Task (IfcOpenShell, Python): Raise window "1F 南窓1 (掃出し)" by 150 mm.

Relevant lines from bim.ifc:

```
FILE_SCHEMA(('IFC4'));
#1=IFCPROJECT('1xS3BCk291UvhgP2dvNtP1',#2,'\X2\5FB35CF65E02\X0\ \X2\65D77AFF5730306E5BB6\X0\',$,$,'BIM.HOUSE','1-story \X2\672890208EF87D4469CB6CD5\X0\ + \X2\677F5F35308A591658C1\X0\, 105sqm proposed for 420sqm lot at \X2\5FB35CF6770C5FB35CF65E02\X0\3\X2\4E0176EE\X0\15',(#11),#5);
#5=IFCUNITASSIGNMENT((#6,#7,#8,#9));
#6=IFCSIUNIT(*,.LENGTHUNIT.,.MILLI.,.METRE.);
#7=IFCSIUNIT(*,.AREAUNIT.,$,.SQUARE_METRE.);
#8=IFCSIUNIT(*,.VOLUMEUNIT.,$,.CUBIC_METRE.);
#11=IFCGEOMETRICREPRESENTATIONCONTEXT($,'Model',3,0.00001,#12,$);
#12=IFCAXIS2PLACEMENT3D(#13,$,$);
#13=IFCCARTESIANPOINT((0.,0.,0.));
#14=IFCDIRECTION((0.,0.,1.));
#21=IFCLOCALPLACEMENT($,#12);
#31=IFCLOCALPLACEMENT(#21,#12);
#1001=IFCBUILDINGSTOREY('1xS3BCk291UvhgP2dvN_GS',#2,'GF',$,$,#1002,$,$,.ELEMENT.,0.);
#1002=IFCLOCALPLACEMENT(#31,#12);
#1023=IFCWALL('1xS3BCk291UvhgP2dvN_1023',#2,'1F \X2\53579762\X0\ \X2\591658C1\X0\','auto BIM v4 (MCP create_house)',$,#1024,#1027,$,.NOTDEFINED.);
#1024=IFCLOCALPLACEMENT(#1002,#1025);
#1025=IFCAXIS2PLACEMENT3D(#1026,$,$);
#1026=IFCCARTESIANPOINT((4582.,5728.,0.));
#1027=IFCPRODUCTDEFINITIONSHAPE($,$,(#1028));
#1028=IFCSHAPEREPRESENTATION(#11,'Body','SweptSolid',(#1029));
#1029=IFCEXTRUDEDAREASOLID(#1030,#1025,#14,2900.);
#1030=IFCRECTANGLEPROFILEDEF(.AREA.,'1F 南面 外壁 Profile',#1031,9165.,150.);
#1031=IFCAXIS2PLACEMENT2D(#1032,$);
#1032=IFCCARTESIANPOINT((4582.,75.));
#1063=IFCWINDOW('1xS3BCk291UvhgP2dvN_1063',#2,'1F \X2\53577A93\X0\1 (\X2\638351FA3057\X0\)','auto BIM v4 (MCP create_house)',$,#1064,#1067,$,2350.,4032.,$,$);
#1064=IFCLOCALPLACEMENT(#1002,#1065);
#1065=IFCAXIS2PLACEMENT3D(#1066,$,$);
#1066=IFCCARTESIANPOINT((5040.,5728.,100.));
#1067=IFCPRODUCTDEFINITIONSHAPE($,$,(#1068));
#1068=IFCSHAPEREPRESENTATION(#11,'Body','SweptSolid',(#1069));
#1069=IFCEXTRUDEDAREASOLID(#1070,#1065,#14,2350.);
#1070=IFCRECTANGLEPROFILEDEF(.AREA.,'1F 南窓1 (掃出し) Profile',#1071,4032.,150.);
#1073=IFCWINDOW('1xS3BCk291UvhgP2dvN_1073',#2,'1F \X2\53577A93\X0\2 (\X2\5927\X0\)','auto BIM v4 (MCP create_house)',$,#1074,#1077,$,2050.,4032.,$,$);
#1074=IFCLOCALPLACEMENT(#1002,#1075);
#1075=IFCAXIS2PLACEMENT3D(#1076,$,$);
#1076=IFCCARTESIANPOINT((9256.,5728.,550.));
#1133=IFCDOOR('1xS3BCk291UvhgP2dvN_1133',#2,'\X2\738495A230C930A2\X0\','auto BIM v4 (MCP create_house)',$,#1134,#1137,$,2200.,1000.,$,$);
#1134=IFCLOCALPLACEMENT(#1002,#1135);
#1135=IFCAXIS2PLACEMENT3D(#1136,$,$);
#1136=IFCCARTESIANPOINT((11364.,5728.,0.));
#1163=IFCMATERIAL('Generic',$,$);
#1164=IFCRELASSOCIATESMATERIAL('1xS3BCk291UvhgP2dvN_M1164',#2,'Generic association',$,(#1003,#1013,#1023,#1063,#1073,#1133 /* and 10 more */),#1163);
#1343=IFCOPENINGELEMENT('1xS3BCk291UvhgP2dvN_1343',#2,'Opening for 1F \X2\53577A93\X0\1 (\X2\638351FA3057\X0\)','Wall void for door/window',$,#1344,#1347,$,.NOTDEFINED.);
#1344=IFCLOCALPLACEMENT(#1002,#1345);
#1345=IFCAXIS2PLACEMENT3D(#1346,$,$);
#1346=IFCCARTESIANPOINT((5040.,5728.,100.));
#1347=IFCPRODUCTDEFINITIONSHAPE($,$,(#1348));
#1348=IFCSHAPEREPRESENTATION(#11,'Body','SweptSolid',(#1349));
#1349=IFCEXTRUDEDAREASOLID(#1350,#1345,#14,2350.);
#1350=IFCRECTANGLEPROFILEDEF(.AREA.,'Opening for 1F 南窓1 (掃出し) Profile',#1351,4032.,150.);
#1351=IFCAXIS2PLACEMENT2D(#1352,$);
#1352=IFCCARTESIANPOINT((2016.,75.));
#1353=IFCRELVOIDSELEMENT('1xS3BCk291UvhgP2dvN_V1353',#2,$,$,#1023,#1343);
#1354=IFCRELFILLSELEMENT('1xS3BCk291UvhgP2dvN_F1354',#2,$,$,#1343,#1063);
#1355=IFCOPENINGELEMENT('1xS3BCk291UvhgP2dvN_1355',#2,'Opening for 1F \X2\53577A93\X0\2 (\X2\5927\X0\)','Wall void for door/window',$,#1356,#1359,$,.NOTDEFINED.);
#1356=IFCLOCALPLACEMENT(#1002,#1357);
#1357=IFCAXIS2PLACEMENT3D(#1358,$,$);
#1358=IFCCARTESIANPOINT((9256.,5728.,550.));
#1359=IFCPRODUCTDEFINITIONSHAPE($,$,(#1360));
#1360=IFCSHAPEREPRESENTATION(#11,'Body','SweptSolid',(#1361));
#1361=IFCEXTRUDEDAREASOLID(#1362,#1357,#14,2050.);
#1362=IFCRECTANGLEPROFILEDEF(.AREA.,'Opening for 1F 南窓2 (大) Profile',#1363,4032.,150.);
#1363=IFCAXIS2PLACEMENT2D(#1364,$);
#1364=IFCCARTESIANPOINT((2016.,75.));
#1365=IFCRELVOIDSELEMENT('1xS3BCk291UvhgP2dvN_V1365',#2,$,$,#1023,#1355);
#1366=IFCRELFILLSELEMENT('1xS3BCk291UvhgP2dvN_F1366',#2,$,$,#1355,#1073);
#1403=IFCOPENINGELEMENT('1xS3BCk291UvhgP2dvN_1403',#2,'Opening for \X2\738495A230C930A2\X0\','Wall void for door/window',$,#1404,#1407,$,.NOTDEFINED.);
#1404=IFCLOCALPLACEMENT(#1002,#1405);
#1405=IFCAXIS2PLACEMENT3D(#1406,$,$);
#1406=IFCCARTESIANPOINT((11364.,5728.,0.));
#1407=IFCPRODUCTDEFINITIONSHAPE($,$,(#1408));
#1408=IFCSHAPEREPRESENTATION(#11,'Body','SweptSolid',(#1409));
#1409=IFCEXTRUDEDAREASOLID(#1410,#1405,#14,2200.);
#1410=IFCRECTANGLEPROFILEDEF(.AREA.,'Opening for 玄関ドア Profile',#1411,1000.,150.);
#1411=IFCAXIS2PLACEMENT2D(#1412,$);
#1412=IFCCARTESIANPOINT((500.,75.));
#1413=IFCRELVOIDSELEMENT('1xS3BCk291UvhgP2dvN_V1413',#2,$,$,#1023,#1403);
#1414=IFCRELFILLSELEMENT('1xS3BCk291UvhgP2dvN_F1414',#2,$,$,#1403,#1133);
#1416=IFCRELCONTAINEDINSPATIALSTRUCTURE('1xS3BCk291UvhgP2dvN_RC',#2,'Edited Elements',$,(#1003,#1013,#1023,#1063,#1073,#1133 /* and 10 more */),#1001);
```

```python
import numpy as np
import ifcopenshell
import ifcopenshell.api.geometry
import ifcopenshell.util.placement
import ifcopenshell.util.unit

model = ifcopenshell.open("bim.ifc")
unit_scale = ifcopenshell.util.unit.calculate_unit_scale(model)

window = model.by_id(1063)
opening = window.FillsVoids[0].RelatingOpeningElement
dz = 0.15 / unit_scale

shift = np.array([0.0, 0.0, dz])
# The window is not placed relative to its opening, so move both.
for product in (opening, window):
    matrix = ifcopenshell.util.placement.get_local_placement(product.ObjectPlacement)
    matrix[:3, 3] += shift
    ifcopenshell.api.geometry.edit_object_placement(model, product=product, matrix=matrix, is_si=False)

print(f"moved by {dz * unit_scale:+.3f} m")

model.write("bim_updated.ifc")
```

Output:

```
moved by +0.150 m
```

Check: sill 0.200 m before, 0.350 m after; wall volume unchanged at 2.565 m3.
